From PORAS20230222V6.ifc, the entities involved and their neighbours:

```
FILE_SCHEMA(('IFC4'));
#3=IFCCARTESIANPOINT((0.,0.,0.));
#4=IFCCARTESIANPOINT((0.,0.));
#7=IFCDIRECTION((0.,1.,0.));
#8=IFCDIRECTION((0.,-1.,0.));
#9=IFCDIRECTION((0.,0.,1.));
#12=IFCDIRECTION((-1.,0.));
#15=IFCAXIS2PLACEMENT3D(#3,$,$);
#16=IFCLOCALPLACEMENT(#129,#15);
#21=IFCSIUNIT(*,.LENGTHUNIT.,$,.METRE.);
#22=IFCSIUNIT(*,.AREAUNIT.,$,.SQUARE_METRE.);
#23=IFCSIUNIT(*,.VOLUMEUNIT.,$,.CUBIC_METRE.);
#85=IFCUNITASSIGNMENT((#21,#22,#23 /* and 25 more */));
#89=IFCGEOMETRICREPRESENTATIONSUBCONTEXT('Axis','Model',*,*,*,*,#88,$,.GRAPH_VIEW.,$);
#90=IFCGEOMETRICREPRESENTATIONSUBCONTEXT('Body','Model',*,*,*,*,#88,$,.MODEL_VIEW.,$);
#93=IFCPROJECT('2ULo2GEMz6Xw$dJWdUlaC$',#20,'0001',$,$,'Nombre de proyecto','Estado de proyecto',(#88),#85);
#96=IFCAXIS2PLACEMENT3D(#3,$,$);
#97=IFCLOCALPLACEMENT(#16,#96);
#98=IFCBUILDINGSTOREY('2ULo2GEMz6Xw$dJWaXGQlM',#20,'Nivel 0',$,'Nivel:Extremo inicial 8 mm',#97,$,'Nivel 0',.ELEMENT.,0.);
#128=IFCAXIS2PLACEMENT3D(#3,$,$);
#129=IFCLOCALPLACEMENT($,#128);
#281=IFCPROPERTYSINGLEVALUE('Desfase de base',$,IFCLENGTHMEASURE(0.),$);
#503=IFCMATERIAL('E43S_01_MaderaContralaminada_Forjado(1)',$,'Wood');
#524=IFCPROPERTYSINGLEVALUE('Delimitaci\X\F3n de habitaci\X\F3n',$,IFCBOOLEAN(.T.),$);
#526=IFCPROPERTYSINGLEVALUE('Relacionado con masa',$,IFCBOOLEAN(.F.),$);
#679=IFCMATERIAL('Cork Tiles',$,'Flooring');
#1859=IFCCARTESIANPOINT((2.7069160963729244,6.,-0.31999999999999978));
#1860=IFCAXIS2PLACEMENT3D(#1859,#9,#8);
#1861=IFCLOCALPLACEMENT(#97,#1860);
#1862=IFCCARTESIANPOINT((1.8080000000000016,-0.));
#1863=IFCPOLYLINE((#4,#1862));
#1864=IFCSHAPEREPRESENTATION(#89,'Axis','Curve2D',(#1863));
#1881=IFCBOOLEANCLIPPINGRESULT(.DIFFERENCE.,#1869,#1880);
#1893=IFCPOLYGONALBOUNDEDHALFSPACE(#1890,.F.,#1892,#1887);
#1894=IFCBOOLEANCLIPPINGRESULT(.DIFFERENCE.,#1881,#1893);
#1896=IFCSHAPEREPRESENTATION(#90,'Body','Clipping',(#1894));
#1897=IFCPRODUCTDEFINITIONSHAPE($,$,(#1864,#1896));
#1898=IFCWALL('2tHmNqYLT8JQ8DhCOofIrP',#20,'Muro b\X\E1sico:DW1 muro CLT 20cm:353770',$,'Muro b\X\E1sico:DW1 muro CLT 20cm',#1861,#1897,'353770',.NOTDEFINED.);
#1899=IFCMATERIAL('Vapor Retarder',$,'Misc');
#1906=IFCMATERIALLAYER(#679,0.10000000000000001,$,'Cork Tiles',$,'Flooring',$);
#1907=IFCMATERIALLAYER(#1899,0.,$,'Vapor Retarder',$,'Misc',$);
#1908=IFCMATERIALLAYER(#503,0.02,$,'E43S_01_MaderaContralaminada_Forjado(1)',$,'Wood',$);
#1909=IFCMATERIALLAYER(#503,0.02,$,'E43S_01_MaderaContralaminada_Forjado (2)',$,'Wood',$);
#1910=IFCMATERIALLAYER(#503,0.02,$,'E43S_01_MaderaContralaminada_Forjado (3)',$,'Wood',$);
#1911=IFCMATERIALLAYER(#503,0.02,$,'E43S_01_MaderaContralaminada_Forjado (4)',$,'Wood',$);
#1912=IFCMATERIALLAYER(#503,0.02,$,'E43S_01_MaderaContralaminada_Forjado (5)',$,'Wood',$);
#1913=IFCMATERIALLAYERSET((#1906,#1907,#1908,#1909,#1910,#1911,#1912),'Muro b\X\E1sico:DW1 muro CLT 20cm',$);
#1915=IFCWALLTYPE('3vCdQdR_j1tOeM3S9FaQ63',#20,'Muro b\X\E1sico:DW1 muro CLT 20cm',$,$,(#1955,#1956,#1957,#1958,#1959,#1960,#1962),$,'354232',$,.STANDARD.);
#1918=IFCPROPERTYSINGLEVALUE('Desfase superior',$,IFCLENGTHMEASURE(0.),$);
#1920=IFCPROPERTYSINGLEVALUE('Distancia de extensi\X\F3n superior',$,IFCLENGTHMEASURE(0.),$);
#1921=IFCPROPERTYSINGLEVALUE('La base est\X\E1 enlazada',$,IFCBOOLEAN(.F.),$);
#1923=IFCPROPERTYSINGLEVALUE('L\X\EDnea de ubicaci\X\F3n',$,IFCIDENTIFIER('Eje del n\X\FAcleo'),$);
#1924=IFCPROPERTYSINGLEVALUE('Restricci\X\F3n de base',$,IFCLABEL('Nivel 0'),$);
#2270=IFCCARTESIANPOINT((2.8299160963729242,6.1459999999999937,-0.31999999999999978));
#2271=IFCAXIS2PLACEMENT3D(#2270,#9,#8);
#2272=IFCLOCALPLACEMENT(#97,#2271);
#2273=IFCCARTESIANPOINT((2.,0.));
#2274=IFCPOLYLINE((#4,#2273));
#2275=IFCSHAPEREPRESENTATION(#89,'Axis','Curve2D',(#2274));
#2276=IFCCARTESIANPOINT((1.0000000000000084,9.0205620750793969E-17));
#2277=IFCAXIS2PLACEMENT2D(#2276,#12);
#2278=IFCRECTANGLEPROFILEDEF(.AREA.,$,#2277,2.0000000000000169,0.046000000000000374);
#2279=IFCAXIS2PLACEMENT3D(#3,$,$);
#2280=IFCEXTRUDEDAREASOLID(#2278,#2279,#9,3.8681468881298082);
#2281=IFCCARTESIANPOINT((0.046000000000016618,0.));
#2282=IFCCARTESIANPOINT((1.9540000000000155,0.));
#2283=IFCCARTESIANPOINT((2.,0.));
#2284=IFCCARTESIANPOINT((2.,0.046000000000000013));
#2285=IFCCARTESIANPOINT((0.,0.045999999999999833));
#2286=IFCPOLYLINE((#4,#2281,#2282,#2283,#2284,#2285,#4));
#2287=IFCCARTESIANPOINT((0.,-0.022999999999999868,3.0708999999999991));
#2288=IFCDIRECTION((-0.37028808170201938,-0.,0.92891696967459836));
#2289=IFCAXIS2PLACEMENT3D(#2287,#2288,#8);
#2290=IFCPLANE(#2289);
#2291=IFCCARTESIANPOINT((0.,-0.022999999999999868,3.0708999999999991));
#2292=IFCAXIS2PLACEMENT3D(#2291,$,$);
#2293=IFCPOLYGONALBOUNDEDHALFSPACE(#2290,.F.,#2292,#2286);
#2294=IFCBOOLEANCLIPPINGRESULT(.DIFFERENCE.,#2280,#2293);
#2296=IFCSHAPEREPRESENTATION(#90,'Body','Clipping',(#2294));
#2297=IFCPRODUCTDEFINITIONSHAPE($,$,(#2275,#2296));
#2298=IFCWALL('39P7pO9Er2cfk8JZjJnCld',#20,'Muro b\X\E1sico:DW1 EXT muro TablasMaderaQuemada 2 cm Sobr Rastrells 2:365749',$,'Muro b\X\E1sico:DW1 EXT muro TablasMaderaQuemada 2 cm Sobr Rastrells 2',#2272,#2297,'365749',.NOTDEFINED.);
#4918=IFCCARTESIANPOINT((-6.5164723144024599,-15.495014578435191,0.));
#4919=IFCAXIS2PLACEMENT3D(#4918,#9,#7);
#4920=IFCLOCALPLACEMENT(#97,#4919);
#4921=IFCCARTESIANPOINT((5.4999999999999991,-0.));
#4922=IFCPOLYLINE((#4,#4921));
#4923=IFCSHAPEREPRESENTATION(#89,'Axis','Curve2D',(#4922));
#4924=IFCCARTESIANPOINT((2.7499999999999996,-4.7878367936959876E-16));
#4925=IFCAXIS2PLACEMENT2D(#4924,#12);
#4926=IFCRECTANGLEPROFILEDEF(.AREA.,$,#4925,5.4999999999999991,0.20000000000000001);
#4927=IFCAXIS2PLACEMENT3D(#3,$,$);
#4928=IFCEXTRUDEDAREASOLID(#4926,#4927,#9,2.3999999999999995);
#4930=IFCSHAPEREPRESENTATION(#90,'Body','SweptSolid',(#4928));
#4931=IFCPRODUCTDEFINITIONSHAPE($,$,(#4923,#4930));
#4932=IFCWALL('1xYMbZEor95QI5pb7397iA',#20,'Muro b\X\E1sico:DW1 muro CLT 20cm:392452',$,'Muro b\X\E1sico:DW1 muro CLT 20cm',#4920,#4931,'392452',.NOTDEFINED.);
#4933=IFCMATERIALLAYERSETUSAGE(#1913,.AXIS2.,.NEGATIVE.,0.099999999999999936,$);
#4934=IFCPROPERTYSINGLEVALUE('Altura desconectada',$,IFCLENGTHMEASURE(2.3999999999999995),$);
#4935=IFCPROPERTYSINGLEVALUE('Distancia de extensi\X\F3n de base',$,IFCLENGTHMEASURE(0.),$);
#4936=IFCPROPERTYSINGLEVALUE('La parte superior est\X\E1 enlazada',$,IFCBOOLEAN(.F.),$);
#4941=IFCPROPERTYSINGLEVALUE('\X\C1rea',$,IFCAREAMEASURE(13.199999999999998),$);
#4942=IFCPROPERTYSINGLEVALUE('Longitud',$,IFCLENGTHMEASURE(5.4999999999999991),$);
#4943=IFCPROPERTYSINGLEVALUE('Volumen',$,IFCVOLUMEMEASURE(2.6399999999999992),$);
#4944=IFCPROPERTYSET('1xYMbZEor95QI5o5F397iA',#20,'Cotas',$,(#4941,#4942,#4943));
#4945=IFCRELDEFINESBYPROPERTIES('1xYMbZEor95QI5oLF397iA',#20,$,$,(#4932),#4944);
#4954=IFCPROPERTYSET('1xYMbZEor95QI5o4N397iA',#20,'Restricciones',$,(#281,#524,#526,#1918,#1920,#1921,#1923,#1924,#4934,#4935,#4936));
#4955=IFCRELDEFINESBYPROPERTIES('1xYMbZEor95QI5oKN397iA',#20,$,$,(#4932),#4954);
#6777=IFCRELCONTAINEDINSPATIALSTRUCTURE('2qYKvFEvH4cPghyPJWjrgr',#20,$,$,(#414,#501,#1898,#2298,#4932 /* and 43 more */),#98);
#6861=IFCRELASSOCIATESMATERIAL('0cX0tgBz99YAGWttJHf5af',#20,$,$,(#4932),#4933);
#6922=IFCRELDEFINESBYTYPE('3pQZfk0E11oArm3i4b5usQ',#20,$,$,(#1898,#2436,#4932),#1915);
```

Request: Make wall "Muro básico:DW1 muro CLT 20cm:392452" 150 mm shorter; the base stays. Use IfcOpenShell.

```python
import ifcopenshell
import ifcopenshell.api.pset
import ifcopenshell.geom
import ifcopenshell.util.element
import ifcopenshell.util.representation
import ifcopenshell.util.shape
import ifcopenshell.util.unit

model = ifcopenshell.open("PORAS20230222V6.ifc")
area_scale = ifcopenshell.util.unit.calculate_unit_scale(model, "AREAUNIT")
volume_scale = ifcopenshell.util.unit.calculate_unit_scale(model, "VOLUMEUNIT")
settings = ifcopenshell.geom.settings()


def volume(element):
    """Net volume in cubic metres, openings subtracted."""
    shape = ifcopenshell.geom.create_shape(settings, element)
    return ifcopenshell.util.shape.get_volume(shape.geometry)


wall = model.by_guid("1xYMbZEor95QI5pb7397iA")
before = volume(wall)

body = ifcopenshell.util.representation.get_representation(wall, "Model", "Body")
solid = body.Items[0]
old_height = solid.Depth
solid.Depth -= 0.15
after = volume(wall)
thickness = 0.2  # wall thickness in metres

# Update the stored height, areas and volumes.
pset = model.by_id(ifcopenshell.util.element.get_pset(wall, "Cotas", should_inherit=False)["id"])
ifcopenshell.api.pset.edit_pset(model, pset=pset, properties={
    "Área": model.create_entity("IfcAreaMeasure", after / thickness / area_scale),
    "Volumen": model.create_entity("IfcVolumeMeasure", after / volume_scale),
})
pset = model.by_id(ifcopenshell.util.element.get_pset(wall, "Restricciones", should_inherit=False)["id"])
ifcopenshell.api.pset.edit_pset(model, pset=pset, properties={
    "Altura desconectada": model.create_entity("IfcLengthMeasure", solid.Depth),
})

print(f"height {old_height:g} -> {solid.Depth:g}, volume {before:.3f} -> {after:.3f} m3")

model.write("PORAS20230222V6_updated.ifc")
```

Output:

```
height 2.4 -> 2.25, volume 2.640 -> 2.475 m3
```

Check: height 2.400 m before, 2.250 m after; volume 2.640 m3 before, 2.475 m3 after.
